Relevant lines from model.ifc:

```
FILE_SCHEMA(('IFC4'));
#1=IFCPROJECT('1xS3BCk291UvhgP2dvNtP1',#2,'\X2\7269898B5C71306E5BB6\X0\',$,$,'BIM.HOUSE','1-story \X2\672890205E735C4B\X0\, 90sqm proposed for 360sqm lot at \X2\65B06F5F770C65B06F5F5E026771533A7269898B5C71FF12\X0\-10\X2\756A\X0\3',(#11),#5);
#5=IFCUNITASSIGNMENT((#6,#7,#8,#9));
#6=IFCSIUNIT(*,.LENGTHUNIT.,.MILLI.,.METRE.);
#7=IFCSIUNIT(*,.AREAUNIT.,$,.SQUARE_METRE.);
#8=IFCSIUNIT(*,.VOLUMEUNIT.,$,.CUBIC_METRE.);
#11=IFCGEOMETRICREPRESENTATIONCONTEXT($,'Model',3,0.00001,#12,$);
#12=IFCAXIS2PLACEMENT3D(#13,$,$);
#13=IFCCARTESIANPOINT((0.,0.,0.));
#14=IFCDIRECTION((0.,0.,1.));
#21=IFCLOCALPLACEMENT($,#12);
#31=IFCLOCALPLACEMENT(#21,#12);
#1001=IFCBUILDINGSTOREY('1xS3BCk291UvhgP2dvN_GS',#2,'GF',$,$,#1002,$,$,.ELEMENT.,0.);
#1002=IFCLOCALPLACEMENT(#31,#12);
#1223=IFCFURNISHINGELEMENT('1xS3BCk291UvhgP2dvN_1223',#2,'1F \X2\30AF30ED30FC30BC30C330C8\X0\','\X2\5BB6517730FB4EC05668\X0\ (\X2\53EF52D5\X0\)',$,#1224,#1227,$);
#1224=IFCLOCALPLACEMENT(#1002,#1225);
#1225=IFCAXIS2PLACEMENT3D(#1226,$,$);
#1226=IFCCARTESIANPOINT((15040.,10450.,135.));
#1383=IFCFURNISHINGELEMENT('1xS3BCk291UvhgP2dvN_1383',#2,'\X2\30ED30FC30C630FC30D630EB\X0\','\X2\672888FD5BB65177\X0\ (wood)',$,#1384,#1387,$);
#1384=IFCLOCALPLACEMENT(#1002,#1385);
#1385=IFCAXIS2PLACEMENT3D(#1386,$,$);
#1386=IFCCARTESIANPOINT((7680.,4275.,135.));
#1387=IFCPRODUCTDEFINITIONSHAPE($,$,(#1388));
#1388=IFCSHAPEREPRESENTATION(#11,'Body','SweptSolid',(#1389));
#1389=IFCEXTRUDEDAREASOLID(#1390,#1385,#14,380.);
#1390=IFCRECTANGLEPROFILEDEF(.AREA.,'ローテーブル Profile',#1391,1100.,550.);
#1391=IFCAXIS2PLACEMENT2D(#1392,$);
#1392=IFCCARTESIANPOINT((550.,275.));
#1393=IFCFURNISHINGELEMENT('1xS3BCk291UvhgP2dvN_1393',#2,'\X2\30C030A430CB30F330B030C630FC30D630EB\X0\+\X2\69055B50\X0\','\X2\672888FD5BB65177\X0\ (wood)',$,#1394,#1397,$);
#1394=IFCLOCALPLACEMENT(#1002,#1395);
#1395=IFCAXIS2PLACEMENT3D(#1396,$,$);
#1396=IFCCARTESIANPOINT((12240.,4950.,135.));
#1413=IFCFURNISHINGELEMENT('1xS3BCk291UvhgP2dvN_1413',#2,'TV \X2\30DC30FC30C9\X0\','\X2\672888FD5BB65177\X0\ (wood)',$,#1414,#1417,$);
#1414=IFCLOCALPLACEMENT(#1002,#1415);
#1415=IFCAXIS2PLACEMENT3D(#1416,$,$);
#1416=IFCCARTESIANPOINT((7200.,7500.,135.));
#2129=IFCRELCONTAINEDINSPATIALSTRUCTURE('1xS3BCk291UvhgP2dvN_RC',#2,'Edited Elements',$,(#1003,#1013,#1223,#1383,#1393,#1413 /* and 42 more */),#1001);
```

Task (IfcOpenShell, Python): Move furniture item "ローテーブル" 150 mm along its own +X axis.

```python
import ifcopenshell
import ifcopenshell.api.geometry
import ifcopenshell.util.placement

model = ifcopenshell.open("model.ifc")

item = model.by_id(1383)
matrix = ifcopenshell.util.placement.get_local_placement(item.ObjectPlacement)
matrix[:3, 3] += matrix[:3, 0] * 150.0
ifcopenshell.api.geometry.edit_object_placement(model, product=item, matrix=matrix, is_si=False)

print(ifcopenshell.util.placement.get_local_placement(item.ObjectPlacement).round(3) + 0.0)

model.write("model_rev.ifc")
```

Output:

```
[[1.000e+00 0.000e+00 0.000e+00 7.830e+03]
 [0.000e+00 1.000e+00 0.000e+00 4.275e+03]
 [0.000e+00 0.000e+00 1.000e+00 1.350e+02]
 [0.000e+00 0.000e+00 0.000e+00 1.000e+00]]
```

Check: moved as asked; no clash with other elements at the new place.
